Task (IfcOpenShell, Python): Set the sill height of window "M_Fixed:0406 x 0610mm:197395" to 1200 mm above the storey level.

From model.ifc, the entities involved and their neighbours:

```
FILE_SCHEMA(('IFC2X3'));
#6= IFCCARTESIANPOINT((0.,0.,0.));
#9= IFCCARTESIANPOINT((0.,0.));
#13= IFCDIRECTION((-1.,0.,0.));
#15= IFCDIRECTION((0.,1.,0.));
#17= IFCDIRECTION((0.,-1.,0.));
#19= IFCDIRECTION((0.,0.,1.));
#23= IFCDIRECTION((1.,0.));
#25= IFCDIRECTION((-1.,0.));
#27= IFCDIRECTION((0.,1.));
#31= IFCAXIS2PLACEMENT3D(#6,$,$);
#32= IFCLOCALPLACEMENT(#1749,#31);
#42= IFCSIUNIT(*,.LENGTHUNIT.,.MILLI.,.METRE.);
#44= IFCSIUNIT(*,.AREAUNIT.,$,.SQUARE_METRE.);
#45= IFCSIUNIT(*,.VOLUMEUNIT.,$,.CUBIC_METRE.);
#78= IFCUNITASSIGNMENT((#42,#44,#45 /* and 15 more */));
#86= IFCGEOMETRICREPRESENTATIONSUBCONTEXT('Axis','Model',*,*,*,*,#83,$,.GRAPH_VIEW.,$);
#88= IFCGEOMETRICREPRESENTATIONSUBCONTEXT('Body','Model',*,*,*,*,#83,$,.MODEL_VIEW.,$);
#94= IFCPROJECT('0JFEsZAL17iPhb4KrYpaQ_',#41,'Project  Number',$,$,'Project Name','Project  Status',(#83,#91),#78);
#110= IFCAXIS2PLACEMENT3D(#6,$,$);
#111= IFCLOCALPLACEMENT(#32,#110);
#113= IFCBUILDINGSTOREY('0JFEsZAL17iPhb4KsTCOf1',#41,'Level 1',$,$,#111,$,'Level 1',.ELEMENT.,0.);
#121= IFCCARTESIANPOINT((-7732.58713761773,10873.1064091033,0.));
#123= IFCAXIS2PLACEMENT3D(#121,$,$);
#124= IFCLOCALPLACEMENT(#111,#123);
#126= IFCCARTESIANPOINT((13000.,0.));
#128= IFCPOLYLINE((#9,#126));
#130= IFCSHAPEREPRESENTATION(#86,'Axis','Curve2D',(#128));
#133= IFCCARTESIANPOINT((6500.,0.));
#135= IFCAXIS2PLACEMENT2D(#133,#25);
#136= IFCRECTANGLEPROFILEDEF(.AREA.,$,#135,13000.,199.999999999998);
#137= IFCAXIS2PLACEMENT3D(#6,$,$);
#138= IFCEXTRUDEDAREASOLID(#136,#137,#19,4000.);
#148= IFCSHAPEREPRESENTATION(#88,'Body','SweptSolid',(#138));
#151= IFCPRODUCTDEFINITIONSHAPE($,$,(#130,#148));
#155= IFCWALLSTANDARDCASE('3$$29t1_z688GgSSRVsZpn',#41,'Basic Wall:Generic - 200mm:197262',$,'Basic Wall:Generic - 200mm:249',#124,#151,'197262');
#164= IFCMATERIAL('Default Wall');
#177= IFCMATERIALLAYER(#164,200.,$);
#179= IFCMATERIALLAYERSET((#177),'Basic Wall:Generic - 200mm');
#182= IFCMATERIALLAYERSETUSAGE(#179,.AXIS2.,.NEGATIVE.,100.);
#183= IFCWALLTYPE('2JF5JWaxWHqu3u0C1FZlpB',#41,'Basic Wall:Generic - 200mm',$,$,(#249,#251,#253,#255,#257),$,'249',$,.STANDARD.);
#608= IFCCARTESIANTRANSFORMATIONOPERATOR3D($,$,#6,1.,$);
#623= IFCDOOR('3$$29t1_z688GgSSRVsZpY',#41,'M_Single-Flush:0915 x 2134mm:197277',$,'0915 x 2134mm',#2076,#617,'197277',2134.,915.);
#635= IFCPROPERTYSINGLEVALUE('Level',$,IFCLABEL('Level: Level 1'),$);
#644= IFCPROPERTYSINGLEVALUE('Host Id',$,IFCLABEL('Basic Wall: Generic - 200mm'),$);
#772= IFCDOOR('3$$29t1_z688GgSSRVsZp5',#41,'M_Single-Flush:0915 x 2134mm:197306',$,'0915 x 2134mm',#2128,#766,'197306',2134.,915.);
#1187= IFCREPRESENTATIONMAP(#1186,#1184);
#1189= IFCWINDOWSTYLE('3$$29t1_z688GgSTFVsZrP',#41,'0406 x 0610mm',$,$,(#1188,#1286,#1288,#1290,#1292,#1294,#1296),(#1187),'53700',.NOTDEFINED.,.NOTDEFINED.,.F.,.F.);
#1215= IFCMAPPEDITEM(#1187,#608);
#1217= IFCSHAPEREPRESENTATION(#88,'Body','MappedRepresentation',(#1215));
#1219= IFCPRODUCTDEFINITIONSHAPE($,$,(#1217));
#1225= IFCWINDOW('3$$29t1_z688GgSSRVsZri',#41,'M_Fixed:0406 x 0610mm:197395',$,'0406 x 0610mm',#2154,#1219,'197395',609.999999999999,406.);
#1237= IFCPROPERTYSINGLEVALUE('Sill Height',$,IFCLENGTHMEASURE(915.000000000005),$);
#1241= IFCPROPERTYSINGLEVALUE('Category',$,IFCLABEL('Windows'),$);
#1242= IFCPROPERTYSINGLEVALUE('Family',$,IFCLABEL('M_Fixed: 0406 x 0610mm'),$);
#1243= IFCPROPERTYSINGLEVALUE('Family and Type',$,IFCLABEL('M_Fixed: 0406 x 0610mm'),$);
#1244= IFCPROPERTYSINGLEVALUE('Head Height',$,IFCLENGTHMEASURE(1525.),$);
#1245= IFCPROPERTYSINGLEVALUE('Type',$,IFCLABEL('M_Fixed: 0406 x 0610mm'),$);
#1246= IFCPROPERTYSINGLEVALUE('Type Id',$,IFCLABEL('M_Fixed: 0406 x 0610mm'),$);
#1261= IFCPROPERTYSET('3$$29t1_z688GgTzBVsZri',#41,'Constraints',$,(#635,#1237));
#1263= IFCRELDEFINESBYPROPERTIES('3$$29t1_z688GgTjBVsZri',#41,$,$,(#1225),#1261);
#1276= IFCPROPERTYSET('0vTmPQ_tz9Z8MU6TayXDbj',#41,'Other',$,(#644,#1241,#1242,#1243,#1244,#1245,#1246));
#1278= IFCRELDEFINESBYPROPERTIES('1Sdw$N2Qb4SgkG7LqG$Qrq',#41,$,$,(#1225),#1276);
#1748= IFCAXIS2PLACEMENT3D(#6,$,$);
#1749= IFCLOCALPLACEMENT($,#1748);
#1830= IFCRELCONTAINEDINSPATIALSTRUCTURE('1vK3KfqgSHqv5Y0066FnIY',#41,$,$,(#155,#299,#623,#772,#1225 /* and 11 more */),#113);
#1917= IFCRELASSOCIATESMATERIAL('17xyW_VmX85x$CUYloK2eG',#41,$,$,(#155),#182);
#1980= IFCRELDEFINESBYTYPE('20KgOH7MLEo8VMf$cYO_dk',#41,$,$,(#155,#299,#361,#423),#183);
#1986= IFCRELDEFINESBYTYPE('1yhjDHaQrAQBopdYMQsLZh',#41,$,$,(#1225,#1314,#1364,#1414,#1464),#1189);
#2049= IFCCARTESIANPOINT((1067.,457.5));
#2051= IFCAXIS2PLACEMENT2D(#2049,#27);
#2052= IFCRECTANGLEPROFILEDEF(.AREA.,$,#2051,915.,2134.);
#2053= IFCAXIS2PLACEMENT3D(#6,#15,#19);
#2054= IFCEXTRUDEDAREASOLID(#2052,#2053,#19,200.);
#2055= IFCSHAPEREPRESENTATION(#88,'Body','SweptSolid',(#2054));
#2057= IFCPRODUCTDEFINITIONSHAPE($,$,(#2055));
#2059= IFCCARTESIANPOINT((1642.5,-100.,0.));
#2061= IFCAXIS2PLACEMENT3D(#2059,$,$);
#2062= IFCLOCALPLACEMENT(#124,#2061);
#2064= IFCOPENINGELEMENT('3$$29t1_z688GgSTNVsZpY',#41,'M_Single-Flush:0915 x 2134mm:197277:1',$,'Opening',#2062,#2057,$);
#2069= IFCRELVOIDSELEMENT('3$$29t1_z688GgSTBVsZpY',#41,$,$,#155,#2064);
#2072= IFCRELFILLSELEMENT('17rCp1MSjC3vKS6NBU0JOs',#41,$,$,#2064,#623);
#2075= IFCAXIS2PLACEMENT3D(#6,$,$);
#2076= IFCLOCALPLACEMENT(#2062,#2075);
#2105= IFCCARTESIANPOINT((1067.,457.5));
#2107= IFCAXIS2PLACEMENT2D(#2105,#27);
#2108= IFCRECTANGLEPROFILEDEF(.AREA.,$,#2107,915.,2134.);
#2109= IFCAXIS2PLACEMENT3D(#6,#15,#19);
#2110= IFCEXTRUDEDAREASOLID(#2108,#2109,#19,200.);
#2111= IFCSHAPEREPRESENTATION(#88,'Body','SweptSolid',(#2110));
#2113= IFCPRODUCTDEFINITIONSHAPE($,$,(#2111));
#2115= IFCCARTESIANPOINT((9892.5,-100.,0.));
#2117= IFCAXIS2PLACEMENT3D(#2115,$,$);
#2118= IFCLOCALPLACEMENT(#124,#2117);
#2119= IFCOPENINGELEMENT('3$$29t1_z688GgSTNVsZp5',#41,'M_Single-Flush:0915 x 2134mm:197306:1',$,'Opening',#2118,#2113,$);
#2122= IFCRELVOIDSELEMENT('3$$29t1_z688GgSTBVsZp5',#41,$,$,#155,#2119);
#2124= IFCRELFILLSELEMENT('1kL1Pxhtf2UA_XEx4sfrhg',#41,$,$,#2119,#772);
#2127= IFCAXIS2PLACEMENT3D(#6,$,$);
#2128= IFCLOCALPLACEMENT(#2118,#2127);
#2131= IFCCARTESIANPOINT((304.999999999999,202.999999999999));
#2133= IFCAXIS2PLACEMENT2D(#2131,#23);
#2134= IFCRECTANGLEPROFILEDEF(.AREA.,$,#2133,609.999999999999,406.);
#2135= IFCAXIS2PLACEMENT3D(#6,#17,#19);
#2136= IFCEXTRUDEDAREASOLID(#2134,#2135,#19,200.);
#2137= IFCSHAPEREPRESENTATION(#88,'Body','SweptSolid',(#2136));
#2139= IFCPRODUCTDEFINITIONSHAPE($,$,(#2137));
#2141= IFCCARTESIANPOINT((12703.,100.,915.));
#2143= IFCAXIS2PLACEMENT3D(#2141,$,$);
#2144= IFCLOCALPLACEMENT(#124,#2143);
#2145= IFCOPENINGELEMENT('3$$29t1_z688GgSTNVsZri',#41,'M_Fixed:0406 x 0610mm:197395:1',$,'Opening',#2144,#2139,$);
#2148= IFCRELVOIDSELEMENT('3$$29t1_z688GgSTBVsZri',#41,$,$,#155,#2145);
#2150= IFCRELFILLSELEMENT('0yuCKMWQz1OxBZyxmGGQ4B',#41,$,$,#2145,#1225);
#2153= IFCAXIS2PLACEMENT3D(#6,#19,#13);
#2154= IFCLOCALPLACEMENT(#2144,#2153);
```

```python
import numpy as np
import ifcopenshell
import ifcopenshell.api.geometry
import ifcopenshell.api.pset
import ifcopenshell.geom
import ifcopenshell.util.element
import ifcopenshell.util.placement
import ifcopenshell.util.shape
import ifcopenshell.util.unit

model = ifcopenshell.open("model.ifc")
unit_scale = ifcopenshell.util.unit.calculate_unit_scale(model)

window = model.by_guid("3$$29t1_z688GgSSRVsZri")
opening = window.FillsVoids[0].RelatingOpeningElement
storey = ifcopenshell.util.element.get_container(window, ifc_class="IfcBuildingStorey")
level = ifcopenshell.util.placement.get_local_placement(storey.ObjectPlacement)[2, 3]

# The opening's origin need not be at the sill, so measure its lowest point.
shape = ifcopenshell.geom.create_shape(ifcopenshell.geom.settings(), opening)
bottom = ifcopenshell.util.shape.get_shape_bottom_elevation(shape, shape.geometry) / unit_scale
dz = level + 1200.0 - bottom

shift = np.array([0.0, 0.0, dz])
# The window is placed relative to its opening, so it follows when the opening moves.
matrix = ifcopenshell.util.placement.get_local_placement(opening.ObjectPlacement)
matrix[:3, 3] += shift
ifcopenshell.api.geometry.edit_object_placement(
    model, product=opening, matrix=matrix, is_si=False, should_transform_children=True
)

# Keep the stored heights in step.
pset = model.by_id(ifcopenshell.util.element.get_pset(window, "Constraints", should_inherit=False)["id"])
ifcopenshell.api.pset.edit_pset(model, pset=pset, properties={
    "Sill Height": model.create_entity("IfcLengthMeasure", ifcopenshell.util.element.get_pset(window, "Constraints", "Sill Height") + dz),
})
pset = model.by_id(ifcopenshell.util.element.get_pset(window, "Other", should_inherit=False)["id"])
ifcopenshell.api.pset.edit_pset(model, pset=pset, properties={
    "Head Height": model.create_entity("IfcLengthMeasure", ifcopenshell.util.element.get_pset(window, "Other", "Head Height") + dz),
})

print(f"moved by {dz * unit_scale:+.3f} m")

model.write("model-out.ifc")
```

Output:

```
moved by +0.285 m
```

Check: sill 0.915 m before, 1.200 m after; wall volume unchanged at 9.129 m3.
